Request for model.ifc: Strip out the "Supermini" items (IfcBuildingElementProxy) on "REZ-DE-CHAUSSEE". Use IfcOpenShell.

First a look at what the model holds.

```python
import ifcopenshell
import ifcopenshell.util.element

model = ifcopenshell.open("model.ifc")
print(model.schema)
storey = next(s for s in model.by_type("IfcBuildingStorey") if s.Name == "REZ-DE-CHAUSSEE")
proxies = [e for e in ifcopenshell.util.element.get_decomposition(storey) if e.is_a("IfcBuildingElementProxy")]
seen = {}
for e in proxies:
    element_type = ifcopenshell.util.element.get_type(e)
    name = element_type.Name if element_type not in (None, e) else None
    seen[name] = seen.get(name, 0) + 1
for name, count in sorted(seen.items(), key=str):
    print(count, "x", name)
```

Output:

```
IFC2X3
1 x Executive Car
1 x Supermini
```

```python
import ifcopenshell
import ifcopenshell.api.root
import ifcopenshell.util.element

model = ifcopenshell.open("model.ifc")

storey = next(s for s in model.by_type("IfcBuildingStorey") if s.Name == "REZ-DE-CHAUSSEE")
proxies = [e for e in ifcopenshell.util.element.get_decomposition(storey) if e.is_a("IfcBuildingElementProxy")]
targets = [e for e in proxies if (t := ifcopenshell.util.element.get_type(e)) not in (None, e) and t.Name == "Supermini"]

for e in targets:
    ifcopenshell.api.root.remove_product(model, product=e)
print(len(targets), "removed")

model.write("model-out.ifc")
```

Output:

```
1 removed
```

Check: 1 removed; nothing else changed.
